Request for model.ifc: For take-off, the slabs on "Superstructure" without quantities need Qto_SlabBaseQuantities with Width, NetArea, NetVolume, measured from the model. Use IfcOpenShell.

First a look at what the model holds.

```python
import ifcopenshell
import ifcopenshell.util.element
import ifcopenshell.util.unit

model = ifcopenshell.open("model.ifc")
print(model.schema)
for unit_type in ("LENGTHUNIT", "AREAUNIT", "VOLUMEUNIT"):
    print(unit_type, ifcopenshell.util.unit.calculate_unit_scale(model, unit_type))
storey = next(s for s in model.by_type("IfcBuildingStorey") if s.Name == "Superstructure")
slabs = [e for e in ifcopenshell.util.element.get_decomposition(storey) if e.is_a("IfcSlab")]
for e in sorted(slabs, key=lambda e: e.id()):
    print(e.id(), e.is_a(), e.Name, list(ifcopenshell.util.element.get_psets(e, qtos_only=True)), sep=" | ")
```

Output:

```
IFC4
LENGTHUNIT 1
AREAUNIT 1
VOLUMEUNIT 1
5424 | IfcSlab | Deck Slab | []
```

```python
import ifcopenshell
import ifcopenshell.api.pset
import ifcopenshell.geom
import ifcopenshell.util.element
import ifcopenshell.util.shape
import ifcopenshell.util.unit

model = ifcopenshell.open("model.ifc")
unit_scale = ifcopenshell.util.unit.calculate_unit_scale(model)
area_scale = ifcopenshell.util.unit.calculate_unit_scale(model, "AREAUNIT")
volume_scale = ifcopenshell.util.unit.calculate_unit_scale(model, "VOLUMEUNIT")
settings = ifcopenshell.geom.settings()

storey = next(s for s in model.by_type("IfcBuildingStorey") if s.Name == "Superstructure")
slabs = [e for e in ifcopenshell.util.element.get_decomposition(storey) if e.is_a("IfcSlab")]

for e in sorted(slabs, key=lambda e: e.id()):
    if ifcopenshell.util.element.get_psets(e, qtos_only=True, should_inherit=False):
        continue
    # Geometry comes back in metres, in the element's own axes.
    shape = ifcopenshell.geom.create_shape(settings, e)
    values = {
        "Width": ifcopenshell.util.shape.get_z(shape.geometry) / unit_scale,
        "NetArea": ifcopenshell.util.shape.get_footprint_area(shape.geometry) / area_scale,
        "NetVolume": ifcopenshell.util.shape.get_volume(shape.geometry) / volume_scale,
    }
    qto = ifcopenshell.api.pset.add_qto(model, product=e, name="Qto_SlabBaseQuantities")
    ifcopenshell.api.pset.edit_qto(model, qto=qto, properties=values)
    print(e.id(), {k: round(v, 3) for k, v in values.items()})

model.write("model-out.ifc")
```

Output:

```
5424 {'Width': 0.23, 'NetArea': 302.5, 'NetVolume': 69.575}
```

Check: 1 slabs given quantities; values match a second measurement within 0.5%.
